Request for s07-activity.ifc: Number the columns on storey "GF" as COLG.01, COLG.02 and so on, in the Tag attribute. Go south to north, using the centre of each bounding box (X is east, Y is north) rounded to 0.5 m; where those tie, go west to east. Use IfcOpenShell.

First a look at what the model holds.

```python
import ifcopenshell
import ifcopenshell.util.element
import ifcopenshell.util.placement

model = ifcopenshell.open("s07-activity.ifc")
print(model.schema)
storey = next(s for s in model.by_type("IfcBuildingStorey") if s.Name == "GF")
columns = [e for e in ifcopenshell.util.element.get_decomposition(storey) if e.is_a("IfcColumn")]
for e in sorted(columns, key=lambda e: e.id()):
    origin = ifcopenshell.util.placement.get_local_placement(e.ObjectPlacement)[:3, 3]
    print(e.id(), e.Tag, e.Name, origin.round(2) + 0.0, sep=" | ")
```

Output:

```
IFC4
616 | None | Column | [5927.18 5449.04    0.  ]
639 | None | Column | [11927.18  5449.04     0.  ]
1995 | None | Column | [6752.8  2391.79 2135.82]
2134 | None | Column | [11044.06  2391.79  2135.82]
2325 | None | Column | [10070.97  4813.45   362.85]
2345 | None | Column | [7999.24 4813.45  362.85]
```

```python
import ifcopenshell
import ifcopenshell.geom
import ifcopenshell.util.element
import ifcopenshell.util.shape

model = ifcopenshell.open("s07-activity.ifc")
settings = ifcopenshell.geom.settings()
settings.set("use-world-coords", True)


def centre(element):
    shape = ifcopenshell.geom.create_shape(settings, element)
    return ifcopenshell.util.shape.get_bbox_centroid(shape.geometry)


storey = next(s for s in model.by_type("IfcBuildingStorey") if s.Name == "GF")
columns = [e for e in ifcopenshell.util.element.get_decomposition(storey) if e.is_a("IfcColumn")]

# Insertion points can sit at a corner or the storey origin, so sort by the geometry (in metres).
centres = {e: centre(e) for e in columns}
columns.sort(key=lambda e: (round(centres[e][1] / 0.5), centres[e][0]))

for i, e in enumerate(columns, start=1):
    number = f"COLG.{i:02d}"
    e.Tag = number
    print(e.id(), number)

model.write("s07-activity_edited.ifc")
```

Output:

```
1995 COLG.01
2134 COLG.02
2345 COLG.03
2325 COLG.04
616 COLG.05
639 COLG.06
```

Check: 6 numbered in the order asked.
